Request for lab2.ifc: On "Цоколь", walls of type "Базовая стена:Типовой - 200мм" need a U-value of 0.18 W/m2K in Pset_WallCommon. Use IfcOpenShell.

First a look at what the model holds.

```python
import ifcopenshell
import ifcopenshell.util.element

model = ifcopenshell.open("lab2.ifc")
print(model.schema)
storey = next(s for s in model.by_type("IfcBuildingStorey") if s.Name == "Цоколь")
walls = [e for e in ifcopenshell.util.element.get_decomposition(storey) if e.is_a("IfcWall")]
seen = {}
for e in walls:
    element_type = ifcopenshell.util.element.get_type(e)
    key = (element_type.Name if element_type != e and element_type else None, ifcopenshell.util.element.get_pset(e, "Pset_WallCommon", "ThermalTransmittance"))
    seen[key] = seen.get(key, 0) + 1
for (name, value), count in sorted(seen.items(), key=str):
    print(count, "x", name, "|", value)
```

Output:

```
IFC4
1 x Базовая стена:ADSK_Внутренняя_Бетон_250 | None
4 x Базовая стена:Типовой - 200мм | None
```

```python
import ifcopenshell
import ifcopenshell.api.pset
import ifcopenshell.util.element

model = ifcopenshell.open("lab2.ifc")

storey = next(s for s in model.by_type("IfcBuildingStorey") if s.Name == "Цоколь")
walls = [e for e in ifcopenshell.util.element.get_decomposition(storey) if e.is_a("IfcWall")]

count = 0
for e in walls:
    element_type = ifcopenshell.util.element.get_type(e)
    if element_type in (None, e) or element_type.Name != "Базовая стена:Типовой - 200мм":
        continue
    # add_pset returns the element's existing set when there is one.
    pset = ifcopenshell.api.pset.add_pset(model, product=e, name="Pset_WallCommon")
    ifcopenshell.api.pset.edit_pset(model, pset=pset, properties={"ThermalTransmittance": 0.18})
    count += 1

print(count, "walls updated")

model.write("lab2_edited.ifc")
```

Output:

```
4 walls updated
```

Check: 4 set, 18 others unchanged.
